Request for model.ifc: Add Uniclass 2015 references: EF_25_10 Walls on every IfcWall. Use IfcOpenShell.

First a look at what the model holds.

```python
import ifcopenshell

model = ifcopenshell.open("model.ifc")
print(model.schema)
print("classifications:", [c.Name for c in model.by_type("IfcClassification")])
for ifc_class in ("IfcDoor", "IfcRoof", "IfcStair", "IfcWall", "IfcWindow"):
    print(ifc_class, len(model.by_type(ifc_class)))
```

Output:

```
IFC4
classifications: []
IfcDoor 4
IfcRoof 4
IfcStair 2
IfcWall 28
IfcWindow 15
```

```python
import ifcopenshell
import ifcopenshell.api.classification

model = ifcopenshell.open("model.ifc")

system = ifcopenshell.api.classification.add_classification(model, classification="Uniclass 2015")

codes = {
    "IfcWall": ("EF_25_10", "Walls"),
}
for ifc_class, (code, name) in codes.items():
    products = model.by_type(ifc_class)
    ifcopenshell.api.classification.add_reference(
        model, products=products, classification=system, identification=code, name=name
    )
    print(code, len(products))

model.write("model-out.ifc")
```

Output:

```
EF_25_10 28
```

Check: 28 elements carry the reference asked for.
